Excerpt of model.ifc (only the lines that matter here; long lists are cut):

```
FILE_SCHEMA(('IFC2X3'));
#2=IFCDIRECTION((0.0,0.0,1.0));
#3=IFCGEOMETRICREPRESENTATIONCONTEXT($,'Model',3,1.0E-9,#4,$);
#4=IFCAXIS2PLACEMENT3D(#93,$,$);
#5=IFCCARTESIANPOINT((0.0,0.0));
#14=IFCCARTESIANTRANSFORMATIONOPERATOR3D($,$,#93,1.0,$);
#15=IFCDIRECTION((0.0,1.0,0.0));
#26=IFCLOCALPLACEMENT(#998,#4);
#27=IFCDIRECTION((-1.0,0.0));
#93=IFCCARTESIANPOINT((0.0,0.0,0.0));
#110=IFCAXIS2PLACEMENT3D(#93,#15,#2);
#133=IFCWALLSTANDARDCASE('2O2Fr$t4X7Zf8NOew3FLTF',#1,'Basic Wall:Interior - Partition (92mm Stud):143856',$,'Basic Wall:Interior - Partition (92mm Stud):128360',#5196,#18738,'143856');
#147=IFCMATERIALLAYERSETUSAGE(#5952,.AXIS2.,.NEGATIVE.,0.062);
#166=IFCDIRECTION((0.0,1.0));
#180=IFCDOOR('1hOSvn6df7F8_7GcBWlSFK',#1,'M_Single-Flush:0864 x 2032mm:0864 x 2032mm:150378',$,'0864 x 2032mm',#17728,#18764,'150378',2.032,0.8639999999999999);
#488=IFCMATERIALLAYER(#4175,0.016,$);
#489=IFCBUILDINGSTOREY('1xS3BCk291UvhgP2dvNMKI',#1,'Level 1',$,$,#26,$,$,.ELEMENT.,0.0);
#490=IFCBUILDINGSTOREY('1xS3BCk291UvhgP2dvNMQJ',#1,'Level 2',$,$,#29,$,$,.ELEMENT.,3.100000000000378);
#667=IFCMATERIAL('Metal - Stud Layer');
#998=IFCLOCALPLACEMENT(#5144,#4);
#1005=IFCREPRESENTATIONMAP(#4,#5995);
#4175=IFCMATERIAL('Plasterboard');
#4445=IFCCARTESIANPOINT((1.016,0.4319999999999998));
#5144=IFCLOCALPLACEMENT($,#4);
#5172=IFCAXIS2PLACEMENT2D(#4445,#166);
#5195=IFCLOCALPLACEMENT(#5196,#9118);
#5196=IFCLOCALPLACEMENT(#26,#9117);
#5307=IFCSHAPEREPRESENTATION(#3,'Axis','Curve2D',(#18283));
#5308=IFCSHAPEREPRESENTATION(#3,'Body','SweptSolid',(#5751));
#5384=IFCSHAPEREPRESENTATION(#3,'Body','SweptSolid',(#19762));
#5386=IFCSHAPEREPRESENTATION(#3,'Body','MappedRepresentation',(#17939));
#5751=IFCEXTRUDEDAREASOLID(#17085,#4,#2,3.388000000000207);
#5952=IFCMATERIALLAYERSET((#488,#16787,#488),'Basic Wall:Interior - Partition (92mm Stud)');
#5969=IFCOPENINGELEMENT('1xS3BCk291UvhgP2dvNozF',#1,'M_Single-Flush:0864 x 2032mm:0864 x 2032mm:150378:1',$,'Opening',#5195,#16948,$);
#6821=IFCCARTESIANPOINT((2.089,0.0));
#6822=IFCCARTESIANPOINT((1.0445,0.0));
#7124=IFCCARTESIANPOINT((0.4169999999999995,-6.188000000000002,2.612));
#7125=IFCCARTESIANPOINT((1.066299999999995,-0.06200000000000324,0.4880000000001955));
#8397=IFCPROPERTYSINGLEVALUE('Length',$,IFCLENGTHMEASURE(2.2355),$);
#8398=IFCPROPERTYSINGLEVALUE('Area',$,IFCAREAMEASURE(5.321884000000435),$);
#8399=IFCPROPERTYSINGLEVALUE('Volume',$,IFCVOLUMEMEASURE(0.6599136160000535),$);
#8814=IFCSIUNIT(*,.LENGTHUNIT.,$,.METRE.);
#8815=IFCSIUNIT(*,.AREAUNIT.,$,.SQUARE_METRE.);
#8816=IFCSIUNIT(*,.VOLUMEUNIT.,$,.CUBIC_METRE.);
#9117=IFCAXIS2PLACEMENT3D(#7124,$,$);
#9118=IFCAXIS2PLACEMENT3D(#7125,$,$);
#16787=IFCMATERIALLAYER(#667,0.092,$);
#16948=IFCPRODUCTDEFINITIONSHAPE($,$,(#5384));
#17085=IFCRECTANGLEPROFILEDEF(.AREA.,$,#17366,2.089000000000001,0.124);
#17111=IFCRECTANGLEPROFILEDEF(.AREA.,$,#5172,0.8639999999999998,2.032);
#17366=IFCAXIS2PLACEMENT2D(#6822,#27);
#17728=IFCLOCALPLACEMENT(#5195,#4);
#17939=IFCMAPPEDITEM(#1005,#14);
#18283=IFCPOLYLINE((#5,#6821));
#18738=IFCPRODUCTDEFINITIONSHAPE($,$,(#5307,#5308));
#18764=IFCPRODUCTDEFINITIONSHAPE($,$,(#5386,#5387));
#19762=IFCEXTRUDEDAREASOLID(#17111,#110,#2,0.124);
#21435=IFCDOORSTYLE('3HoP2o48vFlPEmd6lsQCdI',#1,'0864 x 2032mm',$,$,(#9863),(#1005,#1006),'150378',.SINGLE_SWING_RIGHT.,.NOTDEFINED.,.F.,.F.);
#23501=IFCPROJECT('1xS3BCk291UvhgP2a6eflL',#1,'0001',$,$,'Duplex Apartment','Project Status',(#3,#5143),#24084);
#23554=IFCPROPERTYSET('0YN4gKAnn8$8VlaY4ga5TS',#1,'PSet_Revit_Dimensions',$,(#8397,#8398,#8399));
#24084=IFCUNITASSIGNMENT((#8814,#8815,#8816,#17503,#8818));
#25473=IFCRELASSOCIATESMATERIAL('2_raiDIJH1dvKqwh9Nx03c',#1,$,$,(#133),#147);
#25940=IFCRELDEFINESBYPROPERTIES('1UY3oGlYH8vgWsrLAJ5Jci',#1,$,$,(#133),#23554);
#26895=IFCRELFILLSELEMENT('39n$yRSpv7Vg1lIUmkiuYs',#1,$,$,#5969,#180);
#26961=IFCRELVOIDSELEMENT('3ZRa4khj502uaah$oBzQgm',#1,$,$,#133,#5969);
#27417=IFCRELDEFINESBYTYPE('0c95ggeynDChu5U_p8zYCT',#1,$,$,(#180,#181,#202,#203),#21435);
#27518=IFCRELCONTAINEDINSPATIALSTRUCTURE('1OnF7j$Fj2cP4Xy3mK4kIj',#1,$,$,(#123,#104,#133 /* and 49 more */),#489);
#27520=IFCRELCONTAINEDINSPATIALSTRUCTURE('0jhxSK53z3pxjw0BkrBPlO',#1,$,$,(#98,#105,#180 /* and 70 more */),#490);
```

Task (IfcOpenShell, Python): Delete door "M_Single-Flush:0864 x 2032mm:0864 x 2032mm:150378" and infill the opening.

```python
import ifcopenshell
import ifcopenshell.api.feature
import ifcopenshell.api.pset
import ifcopenshell.api.root
import ifcopenshell.geom
import ifcopenshell.util.element
import ifcopenshell.util.shape
import ifcopenshell.util.unit

model = ifcopenshell.open("model.ifc")
area_scale = ifcopenshell.util.unit.calculate_unit_scale(model, "AREAUNIT")
volume_scale = ifcopenshell.util.unit.calculate_unit_scale(model, "VOLUMEUNIT")
settings = ifcopenshell.geom.settings()


def volume(element):
    """Net volume in cubic metres, openings subtracted."""
    shape = ifcopenshell.geom.create_shape(settings, element)
    return ifcopenshell.util.shape.get_volume(shape.geometry)


door = model.by_guid("1hOSvn6df7F8_7GcBWlSFK")
opening = door.FillsVoids[0].RelatingOpeningElement
wall = opening.VoidsElements[0].RelatingBuildingElement
before = volume(wall)

ifcopenshell.api.root.remove_product(model, product=door)
ifcopenshell.api.feature.remove_feature(model, feature=opening)

after = volume(wall)
thickness = 0.124  # wall thickness in metres

# Update the wall's stored quantities.
pset = model.by_id(ifcopenshell.util.element.get_pset(wall, "PSet_Revit_Dimensions", should_inherit=False)["id"])
ifcopenshell.api.pset.edit_pset(model, pset=pset, properties={
    "Area": model.create_entity("IfcAreaMeasure", after / thickness / area_scale),
    "Volume": model.create_entity("IfcVolumeMeasure", after / volume_scale),
})

print(f"wall volume {before:.3f} -> {after:.3f} m3")

model.write("model_edited.ifc")
```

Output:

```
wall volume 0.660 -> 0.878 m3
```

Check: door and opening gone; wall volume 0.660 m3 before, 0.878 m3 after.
